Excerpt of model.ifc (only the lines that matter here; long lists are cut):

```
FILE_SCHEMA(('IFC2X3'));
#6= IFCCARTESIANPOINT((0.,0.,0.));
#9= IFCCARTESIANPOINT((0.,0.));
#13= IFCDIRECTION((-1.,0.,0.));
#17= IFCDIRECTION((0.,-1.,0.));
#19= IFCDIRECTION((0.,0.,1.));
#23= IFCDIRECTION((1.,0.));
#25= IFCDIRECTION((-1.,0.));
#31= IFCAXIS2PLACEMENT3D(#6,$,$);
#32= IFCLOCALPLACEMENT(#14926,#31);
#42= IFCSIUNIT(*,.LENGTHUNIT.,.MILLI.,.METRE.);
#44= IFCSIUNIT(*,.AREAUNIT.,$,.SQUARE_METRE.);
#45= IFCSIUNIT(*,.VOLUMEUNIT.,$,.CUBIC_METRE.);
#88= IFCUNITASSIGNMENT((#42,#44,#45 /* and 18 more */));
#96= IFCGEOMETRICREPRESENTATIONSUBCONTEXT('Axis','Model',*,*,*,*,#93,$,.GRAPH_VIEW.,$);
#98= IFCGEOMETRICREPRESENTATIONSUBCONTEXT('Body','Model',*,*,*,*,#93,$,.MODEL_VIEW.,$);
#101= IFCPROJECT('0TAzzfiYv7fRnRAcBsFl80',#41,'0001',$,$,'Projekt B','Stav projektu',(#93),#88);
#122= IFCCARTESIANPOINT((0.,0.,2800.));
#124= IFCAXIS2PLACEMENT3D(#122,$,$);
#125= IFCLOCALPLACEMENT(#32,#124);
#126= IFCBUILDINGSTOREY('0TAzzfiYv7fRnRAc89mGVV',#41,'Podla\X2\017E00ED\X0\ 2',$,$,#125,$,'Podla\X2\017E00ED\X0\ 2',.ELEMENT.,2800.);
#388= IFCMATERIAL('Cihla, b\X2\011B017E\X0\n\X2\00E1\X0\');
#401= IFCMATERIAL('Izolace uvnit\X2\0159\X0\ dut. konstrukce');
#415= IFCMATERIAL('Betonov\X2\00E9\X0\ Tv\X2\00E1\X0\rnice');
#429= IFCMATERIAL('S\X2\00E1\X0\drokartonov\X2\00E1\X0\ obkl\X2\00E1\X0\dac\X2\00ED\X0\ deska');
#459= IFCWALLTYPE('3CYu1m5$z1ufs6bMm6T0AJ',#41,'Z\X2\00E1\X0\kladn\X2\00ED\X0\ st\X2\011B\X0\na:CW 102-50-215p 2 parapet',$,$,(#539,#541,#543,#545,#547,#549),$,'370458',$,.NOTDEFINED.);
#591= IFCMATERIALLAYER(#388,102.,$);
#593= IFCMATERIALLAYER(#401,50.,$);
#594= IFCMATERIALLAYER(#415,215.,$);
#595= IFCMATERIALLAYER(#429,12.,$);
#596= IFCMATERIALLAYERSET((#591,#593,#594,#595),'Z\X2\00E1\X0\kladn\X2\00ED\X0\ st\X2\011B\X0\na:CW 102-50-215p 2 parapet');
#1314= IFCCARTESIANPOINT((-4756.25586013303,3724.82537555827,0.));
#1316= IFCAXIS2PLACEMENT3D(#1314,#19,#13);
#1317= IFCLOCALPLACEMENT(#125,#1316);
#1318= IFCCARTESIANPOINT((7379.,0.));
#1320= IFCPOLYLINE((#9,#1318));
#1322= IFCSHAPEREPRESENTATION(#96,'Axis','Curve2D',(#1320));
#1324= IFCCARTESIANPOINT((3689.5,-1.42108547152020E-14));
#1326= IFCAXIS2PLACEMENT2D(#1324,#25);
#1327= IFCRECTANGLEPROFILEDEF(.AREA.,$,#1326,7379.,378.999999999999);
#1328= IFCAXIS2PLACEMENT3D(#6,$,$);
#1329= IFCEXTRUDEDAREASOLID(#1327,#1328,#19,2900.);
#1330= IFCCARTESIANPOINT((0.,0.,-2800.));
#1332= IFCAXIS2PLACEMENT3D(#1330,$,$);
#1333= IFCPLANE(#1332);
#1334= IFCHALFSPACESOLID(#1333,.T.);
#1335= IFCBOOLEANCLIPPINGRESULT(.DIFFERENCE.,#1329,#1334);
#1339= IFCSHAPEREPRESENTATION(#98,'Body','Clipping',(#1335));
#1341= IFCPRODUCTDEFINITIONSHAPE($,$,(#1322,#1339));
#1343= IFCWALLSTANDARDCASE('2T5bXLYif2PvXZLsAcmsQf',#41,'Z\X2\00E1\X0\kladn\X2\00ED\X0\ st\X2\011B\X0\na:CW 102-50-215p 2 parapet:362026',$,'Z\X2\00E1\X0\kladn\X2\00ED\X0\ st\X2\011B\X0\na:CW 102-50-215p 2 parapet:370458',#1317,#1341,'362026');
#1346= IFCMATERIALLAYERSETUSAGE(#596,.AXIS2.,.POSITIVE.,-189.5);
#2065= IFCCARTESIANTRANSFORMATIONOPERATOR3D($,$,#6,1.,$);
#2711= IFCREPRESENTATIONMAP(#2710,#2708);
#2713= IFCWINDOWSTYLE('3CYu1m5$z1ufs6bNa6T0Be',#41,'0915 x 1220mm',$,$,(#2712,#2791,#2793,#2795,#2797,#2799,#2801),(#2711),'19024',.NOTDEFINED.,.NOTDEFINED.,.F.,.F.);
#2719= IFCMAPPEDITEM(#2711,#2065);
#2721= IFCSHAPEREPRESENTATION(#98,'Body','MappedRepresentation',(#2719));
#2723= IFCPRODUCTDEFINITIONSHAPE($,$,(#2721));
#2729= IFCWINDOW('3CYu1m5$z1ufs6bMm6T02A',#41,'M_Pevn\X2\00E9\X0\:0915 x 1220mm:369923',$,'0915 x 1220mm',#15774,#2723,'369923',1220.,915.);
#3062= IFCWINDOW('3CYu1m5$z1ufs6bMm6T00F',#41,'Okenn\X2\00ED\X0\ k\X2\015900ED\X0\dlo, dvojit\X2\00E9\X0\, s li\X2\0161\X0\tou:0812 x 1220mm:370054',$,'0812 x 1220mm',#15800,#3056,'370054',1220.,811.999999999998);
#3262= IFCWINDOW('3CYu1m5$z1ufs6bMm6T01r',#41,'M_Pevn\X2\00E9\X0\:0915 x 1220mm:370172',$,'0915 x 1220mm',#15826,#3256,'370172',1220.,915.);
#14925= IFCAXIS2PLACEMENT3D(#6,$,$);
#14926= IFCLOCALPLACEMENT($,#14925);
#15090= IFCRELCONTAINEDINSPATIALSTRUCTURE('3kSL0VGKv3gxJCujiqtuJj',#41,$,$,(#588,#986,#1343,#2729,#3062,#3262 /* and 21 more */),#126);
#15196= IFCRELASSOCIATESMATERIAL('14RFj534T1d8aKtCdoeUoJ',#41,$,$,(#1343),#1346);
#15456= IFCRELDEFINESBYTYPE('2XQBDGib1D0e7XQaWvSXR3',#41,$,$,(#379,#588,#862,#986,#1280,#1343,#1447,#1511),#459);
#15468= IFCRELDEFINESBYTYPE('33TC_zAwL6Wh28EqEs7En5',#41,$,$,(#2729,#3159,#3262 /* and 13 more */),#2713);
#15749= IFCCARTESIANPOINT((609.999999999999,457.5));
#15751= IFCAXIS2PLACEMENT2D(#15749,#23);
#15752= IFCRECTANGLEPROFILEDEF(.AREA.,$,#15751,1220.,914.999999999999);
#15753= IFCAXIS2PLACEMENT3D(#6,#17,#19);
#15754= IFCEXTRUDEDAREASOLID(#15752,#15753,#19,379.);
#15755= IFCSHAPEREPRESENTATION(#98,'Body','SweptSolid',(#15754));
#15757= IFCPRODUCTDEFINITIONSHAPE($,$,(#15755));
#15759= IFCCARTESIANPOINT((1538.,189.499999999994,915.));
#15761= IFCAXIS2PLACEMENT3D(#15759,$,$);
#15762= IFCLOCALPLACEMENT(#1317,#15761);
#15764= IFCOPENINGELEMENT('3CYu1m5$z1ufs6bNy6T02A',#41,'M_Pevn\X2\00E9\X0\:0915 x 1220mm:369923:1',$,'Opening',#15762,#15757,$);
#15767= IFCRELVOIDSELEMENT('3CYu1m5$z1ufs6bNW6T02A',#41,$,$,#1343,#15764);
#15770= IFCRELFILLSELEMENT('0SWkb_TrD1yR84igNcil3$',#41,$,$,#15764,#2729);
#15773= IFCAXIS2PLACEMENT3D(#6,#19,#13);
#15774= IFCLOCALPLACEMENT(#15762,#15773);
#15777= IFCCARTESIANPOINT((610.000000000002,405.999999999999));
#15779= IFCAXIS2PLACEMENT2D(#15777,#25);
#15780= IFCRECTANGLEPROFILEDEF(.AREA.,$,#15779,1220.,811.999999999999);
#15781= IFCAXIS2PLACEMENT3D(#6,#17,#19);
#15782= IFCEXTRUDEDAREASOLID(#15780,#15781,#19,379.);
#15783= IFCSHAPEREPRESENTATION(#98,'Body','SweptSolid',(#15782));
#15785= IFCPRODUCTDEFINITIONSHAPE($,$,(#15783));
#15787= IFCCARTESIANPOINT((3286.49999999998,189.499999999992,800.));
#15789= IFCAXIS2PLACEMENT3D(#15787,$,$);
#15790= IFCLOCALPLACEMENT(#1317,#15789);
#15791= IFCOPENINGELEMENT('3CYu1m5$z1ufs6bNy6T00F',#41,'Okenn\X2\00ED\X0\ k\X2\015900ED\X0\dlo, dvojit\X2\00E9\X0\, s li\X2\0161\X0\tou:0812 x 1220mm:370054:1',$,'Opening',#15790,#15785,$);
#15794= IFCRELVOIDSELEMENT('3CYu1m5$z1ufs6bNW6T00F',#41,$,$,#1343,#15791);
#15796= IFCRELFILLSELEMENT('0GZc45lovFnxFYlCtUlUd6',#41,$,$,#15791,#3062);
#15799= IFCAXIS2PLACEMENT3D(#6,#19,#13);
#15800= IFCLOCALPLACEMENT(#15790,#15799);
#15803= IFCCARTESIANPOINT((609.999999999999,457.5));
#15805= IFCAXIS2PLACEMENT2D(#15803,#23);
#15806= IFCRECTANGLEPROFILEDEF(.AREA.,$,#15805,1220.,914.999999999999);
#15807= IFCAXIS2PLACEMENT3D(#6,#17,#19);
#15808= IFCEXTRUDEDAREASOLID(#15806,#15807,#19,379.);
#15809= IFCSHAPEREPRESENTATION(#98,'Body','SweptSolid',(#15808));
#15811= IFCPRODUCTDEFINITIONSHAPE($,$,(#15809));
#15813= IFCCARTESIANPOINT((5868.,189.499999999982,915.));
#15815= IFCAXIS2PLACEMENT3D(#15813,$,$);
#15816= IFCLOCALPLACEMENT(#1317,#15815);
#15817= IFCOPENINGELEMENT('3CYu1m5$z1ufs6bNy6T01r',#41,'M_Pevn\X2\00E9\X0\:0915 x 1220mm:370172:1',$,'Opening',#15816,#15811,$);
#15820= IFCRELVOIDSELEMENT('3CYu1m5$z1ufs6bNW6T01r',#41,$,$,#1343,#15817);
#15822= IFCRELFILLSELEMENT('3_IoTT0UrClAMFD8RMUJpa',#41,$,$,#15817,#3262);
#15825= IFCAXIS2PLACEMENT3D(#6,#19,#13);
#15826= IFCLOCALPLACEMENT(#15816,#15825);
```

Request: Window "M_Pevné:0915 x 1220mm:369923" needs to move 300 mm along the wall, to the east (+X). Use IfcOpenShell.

```python
import ifcopenshell
import ifcopenshell.api.geometry
import ifcopenshell.util.placement
import ifcopenshell.util.unit

model = ifcopenshell.open("model.ifc")
unit_scale = ifcopenshell.util.unit.calculate_unit_scale(model)

window = model.by_guid("3CYu1m5$z1ufs6bMm6T02A")
opening = window.FillsVoids[0].RelatingOpeningElement
wall = opening.VoidsElements[0].RelatingBuildingElement

wall_matrix = ifcopenshell.util.placement.get_local_placement(wall.ObjectPlacement)
shift = wall_matrix[:3, 0] * -0.3 / unit_scale
before = ifcopenshell.util.placement.get_local_placement(window.ObjectPlacement)[:3, 3].copy()

# The window is placed relative to its opening, so it follows when the opening moves.
matrix = ifcopenshell.util.placement.get_local_placement(opening.ObjectPlacement)
matrix[:3, 3] += shift
ifcopenshell.api.geometry.edit_object_placement(
    model, product=opening, matrix=matrix, is_si=False, should_transform_children=True
)

after = ifcopenshell.util.placement.get_local_placement(window.ObjectPlacement)[:3, 3]
print("window moved by", (after - before).round(3) + 0.0)

model.write("model_rev.ifc")
```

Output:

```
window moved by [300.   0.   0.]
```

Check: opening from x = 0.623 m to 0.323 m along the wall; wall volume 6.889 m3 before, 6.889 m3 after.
